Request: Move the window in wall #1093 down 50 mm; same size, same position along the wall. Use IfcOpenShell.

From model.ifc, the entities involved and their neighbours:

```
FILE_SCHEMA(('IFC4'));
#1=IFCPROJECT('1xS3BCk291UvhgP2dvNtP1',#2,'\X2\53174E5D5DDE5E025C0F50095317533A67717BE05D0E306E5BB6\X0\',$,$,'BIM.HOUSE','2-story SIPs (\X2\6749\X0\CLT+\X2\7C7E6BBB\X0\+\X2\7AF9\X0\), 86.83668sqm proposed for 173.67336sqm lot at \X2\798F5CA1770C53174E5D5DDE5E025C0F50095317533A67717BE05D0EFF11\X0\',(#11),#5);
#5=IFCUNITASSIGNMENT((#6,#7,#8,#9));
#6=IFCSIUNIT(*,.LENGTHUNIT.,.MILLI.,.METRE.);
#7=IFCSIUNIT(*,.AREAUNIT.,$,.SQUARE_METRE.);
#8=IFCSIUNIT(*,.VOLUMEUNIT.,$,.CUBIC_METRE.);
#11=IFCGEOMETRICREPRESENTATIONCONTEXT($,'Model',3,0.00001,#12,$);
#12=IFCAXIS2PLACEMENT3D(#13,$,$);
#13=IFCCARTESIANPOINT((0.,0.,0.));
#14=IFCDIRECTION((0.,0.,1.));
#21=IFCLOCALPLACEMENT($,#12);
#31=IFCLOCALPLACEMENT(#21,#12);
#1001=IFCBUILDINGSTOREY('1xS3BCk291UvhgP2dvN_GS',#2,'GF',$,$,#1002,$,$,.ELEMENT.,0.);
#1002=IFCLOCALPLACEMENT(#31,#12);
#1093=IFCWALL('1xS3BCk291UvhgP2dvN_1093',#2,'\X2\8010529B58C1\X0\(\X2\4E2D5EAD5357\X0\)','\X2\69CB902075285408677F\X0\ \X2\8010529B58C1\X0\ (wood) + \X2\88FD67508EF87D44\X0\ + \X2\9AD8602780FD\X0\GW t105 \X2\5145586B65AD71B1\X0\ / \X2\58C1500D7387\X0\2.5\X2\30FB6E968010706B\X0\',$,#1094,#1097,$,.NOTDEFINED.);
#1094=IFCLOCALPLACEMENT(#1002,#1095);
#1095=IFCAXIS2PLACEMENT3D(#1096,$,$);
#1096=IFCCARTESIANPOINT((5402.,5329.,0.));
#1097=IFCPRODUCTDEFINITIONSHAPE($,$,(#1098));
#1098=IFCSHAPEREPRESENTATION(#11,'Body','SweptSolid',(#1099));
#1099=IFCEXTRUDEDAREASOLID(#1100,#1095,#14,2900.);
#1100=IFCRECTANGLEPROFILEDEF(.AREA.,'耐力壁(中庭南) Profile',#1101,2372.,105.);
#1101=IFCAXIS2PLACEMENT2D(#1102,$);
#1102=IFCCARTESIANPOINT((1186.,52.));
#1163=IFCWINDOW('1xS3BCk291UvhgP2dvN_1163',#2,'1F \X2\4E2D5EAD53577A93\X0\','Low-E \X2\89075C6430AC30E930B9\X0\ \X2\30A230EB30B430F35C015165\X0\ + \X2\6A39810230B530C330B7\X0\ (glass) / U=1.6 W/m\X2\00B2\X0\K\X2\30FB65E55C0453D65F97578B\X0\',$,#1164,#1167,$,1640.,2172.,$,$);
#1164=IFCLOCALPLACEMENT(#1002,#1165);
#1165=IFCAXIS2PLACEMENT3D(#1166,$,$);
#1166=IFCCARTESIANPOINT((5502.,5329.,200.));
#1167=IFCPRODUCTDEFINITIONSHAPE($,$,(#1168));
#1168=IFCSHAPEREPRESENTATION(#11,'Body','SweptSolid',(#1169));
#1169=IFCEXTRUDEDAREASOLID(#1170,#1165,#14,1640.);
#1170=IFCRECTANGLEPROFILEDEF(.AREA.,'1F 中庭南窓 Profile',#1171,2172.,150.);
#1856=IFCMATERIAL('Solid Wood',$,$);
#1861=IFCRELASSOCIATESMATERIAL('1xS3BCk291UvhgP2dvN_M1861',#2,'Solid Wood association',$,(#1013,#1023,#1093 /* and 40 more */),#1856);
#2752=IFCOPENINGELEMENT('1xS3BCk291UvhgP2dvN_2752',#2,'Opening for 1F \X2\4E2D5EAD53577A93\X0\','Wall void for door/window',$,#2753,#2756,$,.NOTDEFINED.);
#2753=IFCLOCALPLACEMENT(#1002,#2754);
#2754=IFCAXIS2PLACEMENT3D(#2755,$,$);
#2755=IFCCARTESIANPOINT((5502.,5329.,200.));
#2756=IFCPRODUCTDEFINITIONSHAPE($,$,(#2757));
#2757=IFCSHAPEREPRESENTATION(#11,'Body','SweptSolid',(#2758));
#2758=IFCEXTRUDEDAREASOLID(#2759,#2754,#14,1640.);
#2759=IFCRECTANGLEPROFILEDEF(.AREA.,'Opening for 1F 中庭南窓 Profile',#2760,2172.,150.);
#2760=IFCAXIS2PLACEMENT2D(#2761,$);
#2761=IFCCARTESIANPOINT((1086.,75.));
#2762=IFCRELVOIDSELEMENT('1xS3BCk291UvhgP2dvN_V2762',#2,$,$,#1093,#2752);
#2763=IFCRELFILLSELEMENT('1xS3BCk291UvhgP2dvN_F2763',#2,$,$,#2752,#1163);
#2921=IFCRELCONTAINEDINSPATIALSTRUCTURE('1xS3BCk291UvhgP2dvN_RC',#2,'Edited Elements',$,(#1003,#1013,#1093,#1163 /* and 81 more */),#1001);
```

```python
import numpy as np
import ifcopenshell
import ifcopenshell.api.geometry
import ifcopenshell.util.placement
import ifcopenshell.util.unit

model = ifcopenshell.open("model.ifc")
unit_scale = ifcopenshell.util.unit.calculate_unit_scale(model)

window = model.by_id(1163)
opening = window.FillsVoids[0].RelatingOpeningElement
dz = -50.0

shift = np.array([0.0, 0.0, dz])
# The window is not placed relative to its opening, so move both.
for product in (opening, window):
    matrix = ifcopenshell.util.placement.get_local_placement(product.ObjectPlacement)
    matrix[:3, 3] += shift
    ifcopenshell.api.geometry.edit_object_placement(model, product=product, matrix=matrix, is_si=False)

print(f"moved by {dz * unit_scale:+.3f} m")

model.write("model_edited.ifc")
```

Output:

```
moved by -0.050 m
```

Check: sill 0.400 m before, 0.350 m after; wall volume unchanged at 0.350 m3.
